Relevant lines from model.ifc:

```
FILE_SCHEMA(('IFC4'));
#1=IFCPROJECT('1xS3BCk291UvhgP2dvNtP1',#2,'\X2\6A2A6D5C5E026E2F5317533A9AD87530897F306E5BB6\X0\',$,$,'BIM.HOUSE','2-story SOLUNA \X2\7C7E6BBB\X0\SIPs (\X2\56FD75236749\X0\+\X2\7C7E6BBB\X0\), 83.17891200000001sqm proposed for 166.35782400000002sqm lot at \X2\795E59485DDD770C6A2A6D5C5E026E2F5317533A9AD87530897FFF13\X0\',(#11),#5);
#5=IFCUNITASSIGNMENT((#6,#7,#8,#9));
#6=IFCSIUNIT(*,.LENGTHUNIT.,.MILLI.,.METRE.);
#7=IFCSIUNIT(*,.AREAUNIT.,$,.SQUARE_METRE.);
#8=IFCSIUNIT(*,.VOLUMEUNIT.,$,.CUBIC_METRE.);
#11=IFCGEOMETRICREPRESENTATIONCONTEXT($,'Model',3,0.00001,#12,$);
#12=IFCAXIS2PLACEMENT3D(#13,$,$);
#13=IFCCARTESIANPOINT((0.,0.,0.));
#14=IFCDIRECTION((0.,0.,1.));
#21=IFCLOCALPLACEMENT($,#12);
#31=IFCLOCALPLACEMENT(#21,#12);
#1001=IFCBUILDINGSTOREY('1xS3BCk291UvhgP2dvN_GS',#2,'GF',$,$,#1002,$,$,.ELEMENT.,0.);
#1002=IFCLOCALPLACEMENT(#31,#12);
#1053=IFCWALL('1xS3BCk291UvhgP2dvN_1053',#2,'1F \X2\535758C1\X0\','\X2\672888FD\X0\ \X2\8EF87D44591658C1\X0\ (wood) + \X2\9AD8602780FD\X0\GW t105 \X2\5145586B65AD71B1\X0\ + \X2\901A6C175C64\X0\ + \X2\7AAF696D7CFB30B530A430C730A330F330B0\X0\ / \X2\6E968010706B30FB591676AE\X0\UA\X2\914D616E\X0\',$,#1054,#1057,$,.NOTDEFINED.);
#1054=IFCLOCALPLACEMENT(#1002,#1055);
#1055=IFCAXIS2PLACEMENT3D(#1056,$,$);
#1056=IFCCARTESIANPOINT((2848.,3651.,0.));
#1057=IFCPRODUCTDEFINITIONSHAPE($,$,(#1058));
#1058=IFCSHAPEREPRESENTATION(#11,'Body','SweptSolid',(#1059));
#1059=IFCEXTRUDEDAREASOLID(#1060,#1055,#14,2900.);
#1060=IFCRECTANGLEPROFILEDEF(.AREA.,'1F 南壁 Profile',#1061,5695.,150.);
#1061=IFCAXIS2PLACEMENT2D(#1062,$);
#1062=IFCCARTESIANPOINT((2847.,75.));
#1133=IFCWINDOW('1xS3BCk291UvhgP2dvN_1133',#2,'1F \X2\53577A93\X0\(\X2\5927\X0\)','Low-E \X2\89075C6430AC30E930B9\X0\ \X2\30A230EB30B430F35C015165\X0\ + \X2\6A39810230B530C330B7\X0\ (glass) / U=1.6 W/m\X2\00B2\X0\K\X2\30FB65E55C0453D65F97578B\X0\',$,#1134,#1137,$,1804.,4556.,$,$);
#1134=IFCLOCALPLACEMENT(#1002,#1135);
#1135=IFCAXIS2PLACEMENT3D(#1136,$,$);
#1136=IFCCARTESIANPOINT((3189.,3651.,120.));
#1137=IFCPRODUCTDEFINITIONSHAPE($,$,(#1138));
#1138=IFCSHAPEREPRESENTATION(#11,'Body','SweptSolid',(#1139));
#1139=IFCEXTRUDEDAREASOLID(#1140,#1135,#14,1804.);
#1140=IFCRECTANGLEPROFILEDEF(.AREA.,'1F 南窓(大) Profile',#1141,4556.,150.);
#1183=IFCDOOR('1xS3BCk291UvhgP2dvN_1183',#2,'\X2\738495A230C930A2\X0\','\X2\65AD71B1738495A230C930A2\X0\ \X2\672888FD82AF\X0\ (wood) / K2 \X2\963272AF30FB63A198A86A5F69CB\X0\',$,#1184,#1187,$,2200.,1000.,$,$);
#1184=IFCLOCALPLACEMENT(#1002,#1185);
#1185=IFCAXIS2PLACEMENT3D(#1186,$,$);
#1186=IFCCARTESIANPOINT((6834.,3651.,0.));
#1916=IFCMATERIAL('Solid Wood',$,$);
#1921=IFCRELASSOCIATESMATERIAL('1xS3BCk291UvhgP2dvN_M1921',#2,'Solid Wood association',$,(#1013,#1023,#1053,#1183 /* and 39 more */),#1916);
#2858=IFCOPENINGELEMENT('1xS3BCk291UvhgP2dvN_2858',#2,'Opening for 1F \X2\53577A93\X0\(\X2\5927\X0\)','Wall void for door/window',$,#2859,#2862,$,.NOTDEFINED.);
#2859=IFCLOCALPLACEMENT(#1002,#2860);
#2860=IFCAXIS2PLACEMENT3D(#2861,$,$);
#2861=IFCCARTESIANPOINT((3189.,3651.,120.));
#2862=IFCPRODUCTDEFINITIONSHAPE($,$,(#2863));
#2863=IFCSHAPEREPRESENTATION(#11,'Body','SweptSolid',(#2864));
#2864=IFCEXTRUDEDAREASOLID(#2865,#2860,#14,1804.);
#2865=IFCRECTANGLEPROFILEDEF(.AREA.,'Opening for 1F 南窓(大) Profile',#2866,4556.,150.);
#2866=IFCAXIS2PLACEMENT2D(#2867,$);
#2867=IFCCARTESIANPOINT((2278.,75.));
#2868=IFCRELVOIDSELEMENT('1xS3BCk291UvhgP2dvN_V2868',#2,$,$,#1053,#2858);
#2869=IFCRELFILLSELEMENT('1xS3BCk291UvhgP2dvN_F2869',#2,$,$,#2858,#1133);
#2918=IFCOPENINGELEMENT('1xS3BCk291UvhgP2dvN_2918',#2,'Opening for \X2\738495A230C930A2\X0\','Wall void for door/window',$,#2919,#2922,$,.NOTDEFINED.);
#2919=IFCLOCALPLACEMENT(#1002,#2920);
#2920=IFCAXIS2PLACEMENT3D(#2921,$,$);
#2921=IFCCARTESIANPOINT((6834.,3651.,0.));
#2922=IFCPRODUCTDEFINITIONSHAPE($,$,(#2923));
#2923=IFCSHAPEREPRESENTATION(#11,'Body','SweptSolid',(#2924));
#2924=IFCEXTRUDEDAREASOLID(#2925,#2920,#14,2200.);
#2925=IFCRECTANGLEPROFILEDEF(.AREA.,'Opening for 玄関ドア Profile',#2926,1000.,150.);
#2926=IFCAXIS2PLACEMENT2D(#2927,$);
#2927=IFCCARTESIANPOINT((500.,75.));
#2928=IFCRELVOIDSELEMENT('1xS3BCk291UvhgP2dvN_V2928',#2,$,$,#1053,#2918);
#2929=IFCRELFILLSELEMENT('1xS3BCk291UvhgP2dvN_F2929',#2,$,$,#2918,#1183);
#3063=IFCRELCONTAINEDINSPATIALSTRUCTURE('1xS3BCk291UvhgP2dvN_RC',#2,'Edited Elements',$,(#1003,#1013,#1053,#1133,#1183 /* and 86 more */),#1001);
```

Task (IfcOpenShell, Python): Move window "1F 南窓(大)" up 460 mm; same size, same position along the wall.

```python
import numpy as np
import ifcopenshell
import ifcopenshell.api.geometry
import ifcopenshell.util.placement
import ifcopenshell.util.unit

model = ifcopenshell.open("model.ifc")
unit_scale = ifcopenshell.util.unit.calculate_unit_scale(model)

window = model.by_guid("1xS3BCk291UvhgP2dvN_1133")
opening = window.FillsVoids[0].RelatingOpeningElement
dz = 0.46 / unit_scale

shift = np.array([0.0, 0.0, dz])
# The window is not placed relative to its opening, so move both.
for product in (opening, window):
    matrix = ifcopenshell.util.placement.get_local_placement(product.ObjectPlacement)
    matrix[:3, 3] += shift
    ifcopenshell.api.geometry.edit_object_placement(model, product=product, matrix=matrix, is_si=False)

print(f"moved by {dz * unit_scale:+.3f} m")

model.write("model_edited.ifc")
```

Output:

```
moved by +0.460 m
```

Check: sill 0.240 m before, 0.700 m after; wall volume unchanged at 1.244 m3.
